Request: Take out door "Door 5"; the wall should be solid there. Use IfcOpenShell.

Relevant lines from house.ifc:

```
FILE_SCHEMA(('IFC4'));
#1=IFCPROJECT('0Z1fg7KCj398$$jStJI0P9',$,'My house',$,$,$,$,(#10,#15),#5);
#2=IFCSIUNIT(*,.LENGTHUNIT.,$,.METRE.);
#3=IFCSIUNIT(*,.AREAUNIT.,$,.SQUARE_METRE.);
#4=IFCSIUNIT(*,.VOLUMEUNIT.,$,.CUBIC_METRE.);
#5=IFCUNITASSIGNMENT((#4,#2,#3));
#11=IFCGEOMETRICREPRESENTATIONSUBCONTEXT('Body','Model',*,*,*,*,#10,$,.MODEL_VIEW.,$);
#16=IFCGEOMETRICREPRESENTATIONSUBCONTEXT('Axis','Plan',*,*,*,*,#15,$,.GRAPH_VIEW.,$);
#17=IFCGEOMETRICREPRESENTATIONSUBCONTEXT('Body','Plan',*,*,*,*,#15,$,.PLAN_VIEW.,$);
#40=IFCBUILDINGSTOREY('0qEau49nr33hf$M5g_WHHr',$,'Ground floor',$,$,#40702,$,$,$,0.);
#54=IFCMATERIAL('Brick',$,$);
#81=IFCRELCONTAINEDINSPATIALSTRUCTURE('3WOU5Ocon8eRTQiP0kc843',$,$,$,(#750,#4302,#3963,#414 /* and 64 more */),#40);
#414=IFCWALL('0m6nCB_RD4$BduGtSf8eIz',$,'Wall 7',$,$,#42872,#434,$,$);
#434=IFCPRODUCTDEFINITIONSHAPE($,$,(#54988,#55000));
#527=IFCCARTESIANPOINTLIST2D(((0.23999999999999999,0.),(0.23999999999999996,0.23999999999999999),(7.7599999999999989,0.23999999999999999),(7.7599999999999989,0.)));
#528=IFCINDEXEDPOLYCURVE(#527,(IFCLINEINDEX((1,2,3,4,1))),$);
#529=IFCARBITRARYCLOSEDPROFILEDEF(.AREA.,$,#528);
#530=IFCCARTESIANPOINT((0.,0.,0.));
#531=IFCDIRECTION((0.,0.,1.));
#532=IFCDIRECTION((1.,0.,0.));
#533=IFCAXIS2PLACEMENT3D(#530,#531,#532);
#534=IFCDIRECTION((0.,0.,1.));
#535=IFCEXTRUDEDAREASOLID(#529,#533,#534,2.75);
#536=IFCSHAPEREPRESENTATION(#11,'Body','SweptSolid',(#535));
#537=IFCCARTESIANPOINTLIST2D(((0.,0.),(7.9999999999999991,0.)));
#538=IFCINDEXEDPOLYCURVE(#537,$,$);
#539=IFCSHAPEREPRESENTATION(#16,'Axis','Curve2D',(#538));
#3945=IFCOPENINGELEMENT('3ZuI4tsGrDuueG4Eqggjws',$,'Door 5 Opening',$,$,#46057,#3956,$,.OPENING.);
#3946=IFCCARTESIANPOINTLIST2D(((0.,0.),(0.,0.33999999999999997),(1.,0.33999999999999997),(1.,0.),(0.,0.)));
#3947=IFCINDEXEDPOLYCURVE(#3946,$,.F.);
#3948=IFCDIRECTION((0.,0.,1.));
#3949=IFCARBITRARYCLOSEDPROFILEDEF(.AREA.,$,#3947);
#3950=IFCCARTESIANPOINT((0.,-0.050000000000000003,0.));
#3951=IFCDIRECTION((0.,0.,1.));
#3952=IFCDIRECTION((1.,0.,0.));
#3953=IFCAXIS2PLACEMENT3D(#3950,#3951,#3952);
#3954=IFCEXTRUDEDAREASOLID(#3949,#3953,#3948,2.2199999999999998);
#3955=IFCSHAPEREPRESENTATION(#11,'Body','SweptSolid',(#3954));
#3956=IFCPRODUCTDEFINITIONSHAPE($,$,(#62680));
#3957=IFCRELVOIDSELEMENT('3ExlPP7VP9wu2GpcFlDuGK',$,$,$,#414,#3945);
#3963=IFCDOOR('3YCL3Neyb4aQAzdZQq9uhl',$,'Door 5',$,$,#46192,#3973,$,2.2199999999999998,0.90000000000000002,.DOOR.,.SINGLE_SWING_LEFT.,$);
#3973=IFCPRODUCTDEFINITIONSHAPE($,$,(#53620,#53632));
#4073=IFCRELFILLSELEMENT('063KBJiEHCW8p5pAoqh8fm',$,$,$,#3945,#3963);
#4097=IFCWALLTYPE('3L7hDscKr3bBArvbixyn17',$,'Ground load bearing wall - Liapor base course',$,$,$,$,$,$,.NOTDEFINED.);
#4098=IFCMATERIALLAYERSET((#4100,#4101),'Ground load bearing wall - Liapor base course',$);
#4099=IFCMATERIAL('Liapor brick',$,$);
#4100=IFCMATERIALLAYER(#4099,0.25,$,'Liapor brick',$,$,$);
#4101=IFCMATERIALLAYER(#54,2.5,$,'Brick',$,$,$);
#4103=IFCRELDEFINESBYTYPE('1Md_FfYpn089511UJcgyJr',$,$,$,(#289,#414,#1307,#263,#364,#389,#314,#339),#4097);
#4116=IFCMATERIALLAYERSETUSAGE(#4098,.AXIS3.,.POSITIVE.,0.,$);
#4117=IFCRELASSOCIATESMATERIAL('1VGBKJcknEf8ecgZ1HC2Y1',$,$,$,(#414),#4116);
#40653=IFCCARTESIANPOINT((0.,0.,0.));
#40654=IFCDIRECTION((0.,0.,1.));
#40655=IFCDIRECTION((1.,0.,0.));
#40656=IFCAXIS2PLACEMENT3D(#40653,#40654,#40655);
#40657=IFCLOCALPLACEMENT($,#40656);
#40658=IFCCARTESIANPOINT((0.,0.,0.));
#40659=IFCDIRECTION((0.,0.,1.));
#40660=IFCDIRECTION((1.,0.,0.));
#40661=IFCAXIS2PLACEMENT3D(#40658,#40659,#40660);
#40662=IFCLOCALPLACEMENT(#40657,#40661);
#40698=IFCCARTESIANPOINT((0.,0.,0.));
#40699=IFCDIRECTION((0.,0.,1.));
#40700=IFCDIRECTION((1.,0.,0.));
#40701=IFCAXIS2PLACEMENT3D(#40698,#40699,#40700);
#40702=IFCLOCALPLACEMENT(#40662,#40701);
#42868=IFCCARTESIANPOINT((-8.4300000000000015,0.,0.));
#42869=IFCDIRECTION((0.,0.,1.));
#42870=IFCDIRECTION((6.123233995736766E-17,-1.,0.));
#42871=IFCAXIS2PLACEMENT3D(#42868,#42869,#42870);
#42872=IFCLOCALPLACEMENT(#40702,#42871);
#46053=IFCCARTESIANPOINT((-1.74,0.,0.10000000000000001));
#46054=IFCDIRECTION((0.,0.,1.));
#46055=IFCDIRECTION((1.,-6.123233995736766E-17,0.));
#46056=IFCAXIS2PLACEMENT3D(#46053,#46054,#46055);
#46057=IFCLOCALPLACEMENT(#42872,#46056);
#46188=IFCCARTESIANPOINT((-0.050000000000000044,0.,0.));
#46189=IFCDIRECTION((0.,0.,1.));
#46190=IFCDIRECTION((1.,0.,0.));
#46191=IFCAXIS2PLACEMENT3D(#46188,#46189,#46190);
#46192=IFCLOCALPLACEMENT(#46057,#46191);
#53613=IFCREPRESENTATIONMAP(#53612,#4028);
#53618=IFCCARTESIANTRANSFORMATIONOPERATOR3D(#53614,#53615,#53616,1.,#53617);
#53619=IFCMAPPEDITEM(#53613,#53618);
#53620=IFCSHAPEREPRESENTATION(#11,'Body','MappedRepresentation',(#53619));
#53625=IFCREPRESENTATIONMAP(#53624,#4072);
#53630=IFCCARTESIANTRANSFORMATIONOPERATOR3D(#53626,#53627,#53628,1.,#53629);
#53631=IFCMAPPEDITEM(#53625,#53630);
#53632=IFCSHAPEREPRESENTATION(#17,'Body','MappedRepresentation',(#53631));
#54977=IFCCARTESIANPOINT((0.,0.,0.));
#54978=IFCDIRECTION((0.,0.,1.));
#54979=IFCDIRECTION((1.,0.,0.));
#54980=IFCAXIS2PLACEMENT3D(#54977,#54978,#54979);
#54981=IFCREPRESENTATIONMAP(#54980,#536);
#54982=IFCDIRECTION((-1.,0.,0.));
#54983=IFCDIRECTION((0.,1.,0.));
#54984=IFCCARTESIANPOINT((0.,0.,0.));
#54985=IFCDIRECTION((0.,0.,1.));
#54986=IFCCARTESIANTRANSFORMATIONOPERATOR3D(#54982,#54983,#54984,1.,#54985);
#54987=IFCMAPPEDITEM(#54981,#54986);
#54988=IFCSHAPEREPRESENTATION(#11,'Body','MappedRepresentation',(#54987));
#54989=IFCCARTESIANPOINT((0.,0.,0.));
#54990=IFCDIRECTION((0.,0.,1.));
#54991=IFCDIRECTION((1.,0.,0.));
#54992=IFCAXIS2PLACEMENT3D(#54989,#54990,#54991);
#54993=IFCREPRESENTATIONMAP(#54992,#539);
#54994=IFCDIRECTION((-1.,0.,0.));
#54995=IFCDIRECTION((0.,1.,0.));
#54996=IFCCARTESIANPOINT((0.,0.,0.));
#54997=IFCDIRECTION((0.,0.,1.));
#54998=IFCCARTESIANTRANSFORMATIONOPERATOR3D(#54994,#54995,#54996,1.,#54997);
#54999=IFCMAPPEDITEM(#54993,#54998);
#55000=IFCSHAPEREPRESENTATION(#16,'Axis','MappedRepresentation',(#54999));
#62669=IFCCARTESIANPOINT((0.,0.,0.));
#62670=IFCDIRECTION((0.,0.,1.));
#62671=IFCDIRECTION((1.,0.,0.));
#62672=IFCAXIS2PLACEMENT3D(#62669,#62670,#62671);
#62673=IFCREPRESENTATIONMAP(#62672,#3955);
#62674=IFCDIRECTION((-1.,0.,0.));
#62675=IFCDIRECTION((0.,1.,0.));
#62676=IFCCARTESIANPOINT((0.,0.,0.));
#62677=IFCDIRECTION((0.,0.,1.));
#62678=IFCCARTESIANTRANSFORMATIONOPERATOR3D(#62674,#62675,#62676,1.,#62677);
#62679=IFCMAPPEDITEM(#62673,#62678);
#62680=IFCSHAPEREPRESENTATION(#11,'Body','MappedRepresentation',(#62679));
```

```python
import ifcopenshell
import ifcopenshell.api.feature
import ifcopenshell.api.root
import ifcopenshell.geom
import ifcopenshell.util.shape

model = ifcopenshell.open("house.ifc")
settings = ifcopenshell.geom.settings()


def volume(element):
    """Net volume in cubic metres, openings subtracted."""
    shape = ifcopenshell.geom.create_shape(settings, element)
    return ifcopenshell.util.shape.get_volume(shape.geometry)


door = model.by_id(3963)
opening = door.FillsVoids[0].RelatingOpeningElement
wall = opening.VoidsElements[0].RelatingBuildingElement
before = volume(wall)

ifcopenshell.api.root.remove_product(model, product=door)
ifcopenshell.api.feature.remove_feature(model, feature=opening)

after = volume(wall)

print(f"wall volume {before:.3f} -> {after:.3f} m3")

model.write("house_v2.ifc")
```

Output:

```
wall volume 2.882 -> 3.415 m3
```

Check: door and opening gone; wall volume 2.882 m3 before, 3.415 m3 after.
